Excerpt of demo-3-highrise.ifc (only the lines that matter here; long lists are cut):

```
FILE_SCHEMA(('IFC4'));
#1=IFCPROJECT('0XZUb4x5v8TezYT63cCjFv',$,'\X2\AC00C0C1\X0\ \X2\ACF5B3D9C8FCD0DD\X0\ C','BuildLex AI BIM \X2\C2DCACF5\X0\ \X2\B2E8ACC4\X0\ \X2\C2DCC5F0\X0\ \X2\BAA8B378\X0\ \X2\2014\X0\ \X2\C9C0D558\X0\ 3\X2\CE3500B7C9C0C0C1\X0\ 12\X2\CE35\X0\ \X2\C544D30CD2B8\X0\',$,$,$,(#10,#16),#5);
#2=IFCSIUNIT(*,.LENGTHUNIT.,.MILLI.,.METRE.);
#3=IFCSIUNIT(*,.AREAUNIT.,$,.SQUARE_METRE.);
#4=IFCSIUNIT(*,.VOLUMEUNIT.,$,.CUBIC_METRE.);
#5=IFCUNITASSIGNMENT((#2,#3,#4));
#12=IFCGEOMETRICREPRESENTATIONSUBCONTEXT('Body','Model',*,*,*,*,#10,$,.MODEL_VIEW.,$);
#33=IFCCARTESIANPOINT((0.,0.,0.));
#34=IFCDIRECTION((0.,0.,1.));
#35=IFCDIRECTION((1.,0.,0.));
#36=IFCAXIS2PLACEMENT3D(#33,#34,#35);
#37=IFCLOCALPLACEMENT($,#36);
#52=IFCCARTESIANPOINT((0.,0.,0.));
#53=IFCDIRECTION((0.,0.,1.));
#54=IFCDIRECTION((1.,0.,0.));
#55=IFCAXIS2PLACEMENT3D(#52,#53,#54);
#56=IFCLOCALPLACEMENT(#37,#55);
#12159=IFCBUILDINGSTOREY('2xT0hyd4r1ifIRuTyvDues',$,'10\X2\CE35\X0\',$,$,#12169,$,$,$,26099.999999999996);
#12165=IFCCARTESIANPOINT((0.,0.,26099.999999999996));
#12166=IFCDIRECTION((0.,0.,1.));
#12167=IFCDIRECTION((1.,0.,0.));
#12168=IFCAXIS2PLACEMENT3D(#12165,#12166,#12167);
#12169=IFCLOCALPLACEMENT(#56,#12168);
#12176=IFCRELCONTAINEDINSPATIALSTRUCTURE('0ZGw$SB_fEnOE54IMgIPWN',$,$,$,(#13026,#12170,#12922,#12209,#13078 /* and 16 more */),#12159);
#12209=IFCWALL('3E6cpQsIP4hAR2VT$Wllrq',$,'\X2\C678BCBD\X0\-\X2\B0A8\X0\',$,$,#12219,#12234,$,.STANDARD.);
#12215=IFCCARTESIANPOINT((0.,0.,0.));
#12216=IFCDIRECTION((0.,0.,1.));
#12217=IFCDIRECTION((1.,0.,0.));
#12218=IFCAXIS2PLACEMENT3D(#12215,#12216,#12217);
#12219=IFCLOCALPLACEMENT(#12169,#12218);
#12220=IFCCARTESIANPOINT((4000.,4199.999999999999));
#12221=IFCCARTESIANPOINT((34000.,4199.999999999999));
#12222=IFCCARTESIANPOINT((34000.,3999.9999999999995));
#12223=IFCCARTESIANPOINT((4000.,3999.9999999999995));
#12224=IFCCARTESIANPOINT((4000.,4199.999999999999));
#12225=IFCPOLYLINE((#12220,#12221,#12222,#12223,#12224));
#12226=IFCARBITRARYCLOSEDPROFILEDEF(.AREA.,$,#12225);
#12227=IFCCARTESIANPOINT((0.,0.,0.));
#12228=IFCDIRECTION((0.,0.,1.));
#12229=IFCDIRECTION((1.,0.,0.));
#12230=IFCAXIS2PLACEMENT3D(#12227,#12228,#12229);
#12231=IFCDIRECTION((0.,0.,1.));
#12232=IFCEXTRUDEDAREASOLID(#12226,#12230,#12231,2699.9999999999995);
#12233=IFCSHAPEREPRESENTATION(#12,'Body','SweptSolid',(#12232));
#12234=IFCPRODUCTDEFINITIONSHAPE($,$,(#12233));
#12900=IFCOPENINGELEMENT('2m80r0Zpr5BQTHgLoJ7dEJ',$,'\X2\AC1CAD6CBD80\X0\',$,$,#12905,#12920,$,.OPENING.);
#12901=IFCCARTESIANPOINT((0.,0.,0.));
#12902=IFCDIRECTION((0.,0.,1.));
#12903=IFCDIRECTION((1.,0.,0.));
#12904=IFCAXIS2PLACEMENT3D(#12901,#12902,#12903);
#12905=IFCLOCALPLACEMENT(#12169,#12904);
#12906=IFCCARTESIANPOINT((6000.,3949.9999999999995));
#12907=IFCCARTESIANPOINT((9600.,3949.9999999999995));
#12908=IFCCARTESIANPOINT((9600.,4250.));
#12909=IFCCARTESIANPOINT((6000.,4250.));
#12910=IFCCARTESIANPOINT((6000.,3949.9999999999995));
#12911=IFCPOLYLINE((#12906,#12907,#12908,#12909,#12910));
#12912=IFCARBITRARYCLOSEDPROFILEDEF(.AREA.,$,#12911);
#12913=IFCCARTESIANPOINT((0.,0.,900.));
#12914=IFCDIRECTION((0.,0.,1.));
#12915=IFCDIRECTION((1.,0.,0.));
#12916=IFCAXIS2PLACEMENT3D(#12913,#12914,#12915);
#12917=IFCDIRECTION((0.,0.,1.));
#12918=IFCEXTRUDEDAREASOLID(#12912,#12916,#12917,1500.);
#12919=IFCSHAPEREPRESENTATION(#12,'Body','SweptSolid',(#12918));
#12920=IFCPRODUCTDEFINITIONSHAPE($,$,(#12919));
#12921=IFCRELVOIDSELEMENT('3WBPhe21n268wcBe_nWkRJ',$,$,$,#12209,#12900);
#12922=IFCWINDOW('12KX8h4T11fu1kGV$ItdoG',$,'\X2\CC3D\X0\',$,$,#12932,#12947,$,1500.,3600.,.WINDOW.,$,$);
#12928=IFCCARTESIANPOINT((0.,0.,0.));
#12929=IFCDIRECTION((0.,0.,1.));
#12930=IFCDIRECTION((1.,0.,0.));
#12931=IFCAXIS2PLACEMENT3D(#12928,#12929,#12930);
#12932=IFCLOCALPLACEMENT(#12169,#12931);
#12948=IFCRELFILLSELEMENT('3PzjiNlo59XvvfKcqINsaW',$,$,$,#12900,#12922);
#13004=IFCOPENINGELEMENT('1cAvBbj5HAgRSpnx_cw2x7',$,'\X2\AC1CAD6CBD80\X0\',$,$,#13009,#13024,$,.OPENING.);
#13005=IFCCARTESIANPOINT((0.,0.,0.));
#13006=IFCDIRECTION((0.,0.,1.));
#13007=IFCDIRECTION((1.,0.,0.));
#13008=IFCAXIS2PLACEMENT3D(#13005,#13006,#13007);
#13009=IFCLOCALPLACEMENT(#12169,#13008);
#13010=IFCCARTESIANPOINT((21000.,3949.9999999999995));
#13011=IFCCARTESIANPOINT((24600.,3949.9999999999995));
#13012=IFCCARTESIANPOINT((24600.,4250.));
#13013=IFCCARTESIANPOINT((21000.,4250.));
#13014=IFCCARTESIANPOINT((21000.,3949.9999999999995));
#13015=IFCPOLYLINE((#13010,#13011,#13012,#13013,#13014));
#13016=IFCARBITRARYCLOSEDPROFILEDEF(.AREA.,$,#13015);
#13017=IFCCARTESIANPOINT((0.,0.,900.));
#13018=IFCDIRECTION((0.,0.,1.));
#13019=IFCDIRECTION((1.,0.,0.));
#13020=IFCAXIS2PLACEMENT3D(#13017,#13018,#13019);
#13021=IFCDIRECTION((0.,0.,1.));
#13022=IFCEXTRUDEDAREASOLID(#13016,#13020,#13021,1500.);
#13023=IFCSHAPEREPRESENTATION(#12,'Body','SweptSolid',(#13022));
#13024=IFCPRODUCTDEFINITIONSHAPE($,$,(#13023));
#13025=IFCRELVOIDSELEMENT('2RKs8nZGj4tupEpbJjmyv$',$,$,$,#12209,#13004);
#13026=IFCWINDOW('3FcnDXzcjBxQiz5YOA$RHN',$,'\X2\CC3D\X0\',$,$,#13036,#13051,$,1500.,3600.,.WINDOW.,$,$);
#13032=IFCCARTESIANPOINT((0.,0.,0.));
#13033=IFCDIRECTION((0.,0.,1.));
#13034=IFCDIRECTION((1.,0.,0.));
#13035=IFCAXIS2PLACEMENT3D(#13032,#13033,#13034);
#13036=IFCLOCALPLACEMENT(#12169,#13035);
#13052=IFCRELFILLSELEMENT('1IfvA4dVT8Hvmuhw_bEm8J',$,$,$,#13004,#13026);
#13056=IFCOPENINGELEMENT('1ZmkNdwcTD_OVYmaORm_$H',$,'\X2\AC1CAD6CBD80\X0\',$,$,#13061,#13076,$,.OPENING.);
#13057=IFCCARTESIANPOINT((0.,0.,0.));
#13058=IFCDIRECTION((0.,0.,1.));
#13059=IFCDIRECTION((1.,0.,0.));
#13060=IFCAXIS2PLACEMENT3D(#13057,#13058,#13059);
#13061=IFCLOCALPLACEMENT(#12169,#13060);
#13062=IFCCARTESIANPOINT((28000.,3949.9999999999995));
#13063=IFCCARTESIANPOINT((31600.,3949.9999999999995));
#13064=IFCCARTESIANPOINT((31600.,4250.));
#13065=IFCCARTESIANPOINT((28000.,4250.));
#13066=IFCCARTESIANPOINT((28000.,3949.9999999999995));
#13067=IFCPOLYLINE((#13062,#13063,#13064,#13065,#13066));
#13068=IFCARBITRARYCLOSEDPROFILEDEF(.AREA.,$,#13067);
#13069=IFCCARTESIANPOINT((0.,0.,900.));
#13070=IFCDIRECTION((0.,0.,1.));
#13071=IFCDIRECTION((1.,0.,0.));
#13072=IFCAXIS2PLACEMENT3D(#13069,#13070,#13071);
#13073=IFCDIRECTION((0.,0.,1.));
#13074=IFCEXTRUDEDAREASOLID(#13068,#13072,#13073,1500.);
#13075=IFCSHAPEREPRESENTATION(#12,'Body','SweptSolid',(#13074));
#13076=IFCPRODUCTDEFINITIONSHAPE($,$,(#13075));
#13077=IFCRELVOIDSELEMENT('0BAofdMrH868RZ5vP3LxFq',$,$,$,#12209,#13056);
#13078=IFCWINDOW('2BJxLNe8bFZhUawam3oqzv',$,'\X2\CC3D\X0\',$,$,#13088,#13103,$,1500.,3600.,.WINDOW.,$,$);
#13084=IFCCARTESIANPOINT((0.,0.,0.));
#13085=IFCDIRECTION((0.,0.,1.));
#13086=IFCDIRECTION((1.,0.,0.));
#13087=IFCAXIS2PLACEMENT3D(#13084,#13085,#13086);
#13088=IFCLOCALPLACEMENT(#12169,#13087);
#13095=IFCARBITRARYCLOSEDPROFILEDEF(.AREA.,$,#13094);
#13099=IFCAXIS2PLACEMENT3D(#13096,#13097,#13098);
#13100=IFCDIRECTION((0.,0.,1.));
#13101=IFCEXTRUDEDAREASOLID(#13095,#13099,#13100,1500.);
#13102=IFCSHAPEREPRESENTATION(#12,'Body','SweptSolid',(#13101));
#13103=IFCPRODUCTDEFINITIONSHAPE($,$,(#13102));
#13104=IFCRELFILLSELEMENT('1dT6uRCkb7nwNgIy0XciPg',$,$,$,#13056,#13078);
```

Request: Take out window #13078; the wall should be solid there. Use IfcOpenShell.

```python
import ifcopenshell
import ifcopenshell.api.feature
import ifcopenshell.api.root
import ifcopenshell.geom
import ifcopenshell.util.shape

model = ifcopenshell.open("demo-3-highrise.ifc")
settings = ifcopenshell.geom.settings()


def volume(element):
    """Net volume in cubic metres, openings subtracted."""
    shape = ifcopenshell.geom.create_shape(settings, element)
    return ifcopenshell.util.shape.get_volume(shape.geometry)


window = model.by_guid("2BJxLNe8bFZhUawam3oqzv")
opening = window.FillsVoids[0].RelatingOpeningElement
wall = opening.VoidsElements[0].RelatingBuildingElement
before = volume(wall)

ifcopenshell.api.root.remove_product(model, product=window)
ifcopenshell.api.feature.remove_feature(model, feature=opening)

after = volume(wall)

print(f"wall volume {before:.3f} -> {after:.3f} m3")

model.write("demo-3-highrise_rev.ifc")
```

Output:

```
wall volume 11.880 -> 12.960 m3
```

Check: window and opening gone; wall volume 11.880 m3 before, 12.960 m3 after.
